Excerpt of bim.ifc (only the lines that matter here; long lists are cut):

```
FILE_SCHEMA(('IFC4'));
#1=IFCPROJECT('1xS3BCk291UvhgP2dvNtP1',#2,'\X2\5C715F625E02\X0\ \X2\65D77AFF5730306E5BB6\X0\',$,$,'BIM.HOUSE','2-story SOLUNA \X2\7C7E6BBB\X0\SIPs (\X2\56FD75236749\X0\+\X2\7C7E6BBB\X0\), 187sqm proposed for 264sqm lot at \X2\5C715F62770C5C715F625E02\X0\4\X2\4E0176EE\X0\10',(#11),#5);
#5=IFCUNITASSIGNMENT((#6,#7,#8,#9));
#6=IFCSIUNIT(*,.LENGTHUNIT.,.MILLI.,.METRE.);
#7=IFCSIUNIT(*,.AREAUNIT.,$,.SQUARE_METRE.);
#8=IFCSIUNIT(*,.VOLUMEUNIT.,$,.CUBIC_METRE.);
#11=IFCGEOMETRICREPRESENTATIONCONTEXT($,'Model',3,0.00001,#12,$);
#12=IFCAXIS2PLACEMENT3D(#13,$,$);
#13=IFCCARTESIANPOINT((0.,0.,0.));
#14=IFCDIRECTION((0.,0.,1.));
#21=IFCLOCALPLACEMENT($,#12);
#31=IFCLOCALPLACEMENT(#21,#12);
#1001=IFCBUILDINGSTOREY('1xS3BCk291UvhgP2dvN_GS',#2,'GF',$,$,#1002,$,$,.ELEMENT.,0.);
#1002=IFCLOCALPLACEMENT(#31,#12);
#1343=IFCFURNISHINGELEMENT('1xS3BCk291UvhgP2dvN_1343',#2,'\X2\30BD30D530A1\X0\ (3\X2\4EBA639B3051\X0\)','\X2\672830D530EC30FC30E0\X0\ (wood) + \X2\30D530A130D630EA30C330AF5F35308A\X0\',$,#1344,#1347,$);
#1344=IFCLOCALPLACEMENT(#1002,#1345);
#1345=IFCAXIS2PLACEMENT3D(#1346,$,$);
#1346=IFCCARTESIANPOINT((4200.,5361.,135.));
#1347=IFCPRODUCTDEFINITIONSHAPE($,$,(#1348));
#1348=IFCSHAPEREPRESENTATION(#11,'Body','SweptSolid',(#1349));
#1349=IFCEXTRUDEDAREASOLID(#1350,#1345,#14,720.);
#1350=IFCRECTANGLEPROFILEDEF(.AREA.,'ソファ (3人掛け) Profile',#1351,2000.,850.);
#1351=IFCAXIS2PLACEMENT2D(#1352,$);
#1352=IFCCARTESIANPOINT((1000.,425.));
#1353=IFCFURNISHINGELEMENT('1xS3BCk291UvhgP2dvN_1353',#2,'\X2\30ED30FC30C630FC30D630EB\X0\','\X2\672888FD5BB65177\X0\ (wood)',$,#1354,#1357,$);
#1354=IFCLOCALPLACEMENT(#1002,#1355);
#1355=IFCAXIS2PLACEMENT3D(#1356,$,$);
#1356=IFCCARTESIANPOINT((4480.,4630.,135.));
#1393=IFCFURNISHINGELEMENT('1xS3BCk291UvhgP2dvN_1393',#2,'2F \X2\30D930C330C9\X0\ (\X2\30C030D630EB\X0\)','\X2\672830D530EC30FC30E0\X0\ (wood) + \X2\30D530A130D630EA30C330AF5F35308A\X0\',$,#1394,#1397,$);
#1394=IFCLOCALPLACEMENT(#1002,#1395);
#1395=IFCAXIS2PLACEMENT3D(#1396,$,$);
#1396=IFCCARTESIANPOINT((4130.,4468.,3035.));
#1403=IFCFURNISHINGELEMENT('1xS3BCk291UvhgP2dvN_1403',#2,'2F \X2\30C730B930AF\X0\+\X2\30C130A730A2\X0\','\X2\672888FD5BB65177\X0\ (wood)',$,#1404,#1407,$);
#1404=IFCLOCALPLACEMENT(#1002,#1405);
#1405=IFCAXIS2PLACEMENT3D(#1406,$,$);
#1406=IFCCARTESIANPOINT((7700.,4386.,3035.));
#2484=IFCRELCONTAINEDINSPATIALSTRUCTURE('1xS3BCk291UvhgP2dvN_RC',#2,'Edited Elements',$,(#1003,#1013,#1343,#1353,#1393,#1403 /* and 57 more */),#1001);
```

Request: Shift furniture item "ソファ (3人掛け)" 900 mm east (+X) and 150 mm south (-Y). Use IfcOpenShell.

```python
import ifcopenshell
import ifcopenshell.api.geometry
import ifcopenshell.util.placement
import ifcopenshell.util.unit

model = ifcopenshell.open("bim.ifc")
unit_scale = ifcopenshell.util.unit.calculate_unit_scale(model)

item = model.by_guid("1xS3BCk291UvhgP2dvN_1343")
matrix = ifcopenshell.util.placement.get_local_placement(item.ObjectPlacement)
matrix[0, 3] += 0.9 / unit_scale
matrix[1, 3] -= 0.15 / unit_scale
ifcopenshell.api.geometry.edit_object_placement(model, product=item, matrix=matrix, is_si=False)

print(ifcopenshell.util.placement.get_local_placement(item.ObjectPlacement).round(3) + 0.0)

model.write("bim_rev.ifc")
```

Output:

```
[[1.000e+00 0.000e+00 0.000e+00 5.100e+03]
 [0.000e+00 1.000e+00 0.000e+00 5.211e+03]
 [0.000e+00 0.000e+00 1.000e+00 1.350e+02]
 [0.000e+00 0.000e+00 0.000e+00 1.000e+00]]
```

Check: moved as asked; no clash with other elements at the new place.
